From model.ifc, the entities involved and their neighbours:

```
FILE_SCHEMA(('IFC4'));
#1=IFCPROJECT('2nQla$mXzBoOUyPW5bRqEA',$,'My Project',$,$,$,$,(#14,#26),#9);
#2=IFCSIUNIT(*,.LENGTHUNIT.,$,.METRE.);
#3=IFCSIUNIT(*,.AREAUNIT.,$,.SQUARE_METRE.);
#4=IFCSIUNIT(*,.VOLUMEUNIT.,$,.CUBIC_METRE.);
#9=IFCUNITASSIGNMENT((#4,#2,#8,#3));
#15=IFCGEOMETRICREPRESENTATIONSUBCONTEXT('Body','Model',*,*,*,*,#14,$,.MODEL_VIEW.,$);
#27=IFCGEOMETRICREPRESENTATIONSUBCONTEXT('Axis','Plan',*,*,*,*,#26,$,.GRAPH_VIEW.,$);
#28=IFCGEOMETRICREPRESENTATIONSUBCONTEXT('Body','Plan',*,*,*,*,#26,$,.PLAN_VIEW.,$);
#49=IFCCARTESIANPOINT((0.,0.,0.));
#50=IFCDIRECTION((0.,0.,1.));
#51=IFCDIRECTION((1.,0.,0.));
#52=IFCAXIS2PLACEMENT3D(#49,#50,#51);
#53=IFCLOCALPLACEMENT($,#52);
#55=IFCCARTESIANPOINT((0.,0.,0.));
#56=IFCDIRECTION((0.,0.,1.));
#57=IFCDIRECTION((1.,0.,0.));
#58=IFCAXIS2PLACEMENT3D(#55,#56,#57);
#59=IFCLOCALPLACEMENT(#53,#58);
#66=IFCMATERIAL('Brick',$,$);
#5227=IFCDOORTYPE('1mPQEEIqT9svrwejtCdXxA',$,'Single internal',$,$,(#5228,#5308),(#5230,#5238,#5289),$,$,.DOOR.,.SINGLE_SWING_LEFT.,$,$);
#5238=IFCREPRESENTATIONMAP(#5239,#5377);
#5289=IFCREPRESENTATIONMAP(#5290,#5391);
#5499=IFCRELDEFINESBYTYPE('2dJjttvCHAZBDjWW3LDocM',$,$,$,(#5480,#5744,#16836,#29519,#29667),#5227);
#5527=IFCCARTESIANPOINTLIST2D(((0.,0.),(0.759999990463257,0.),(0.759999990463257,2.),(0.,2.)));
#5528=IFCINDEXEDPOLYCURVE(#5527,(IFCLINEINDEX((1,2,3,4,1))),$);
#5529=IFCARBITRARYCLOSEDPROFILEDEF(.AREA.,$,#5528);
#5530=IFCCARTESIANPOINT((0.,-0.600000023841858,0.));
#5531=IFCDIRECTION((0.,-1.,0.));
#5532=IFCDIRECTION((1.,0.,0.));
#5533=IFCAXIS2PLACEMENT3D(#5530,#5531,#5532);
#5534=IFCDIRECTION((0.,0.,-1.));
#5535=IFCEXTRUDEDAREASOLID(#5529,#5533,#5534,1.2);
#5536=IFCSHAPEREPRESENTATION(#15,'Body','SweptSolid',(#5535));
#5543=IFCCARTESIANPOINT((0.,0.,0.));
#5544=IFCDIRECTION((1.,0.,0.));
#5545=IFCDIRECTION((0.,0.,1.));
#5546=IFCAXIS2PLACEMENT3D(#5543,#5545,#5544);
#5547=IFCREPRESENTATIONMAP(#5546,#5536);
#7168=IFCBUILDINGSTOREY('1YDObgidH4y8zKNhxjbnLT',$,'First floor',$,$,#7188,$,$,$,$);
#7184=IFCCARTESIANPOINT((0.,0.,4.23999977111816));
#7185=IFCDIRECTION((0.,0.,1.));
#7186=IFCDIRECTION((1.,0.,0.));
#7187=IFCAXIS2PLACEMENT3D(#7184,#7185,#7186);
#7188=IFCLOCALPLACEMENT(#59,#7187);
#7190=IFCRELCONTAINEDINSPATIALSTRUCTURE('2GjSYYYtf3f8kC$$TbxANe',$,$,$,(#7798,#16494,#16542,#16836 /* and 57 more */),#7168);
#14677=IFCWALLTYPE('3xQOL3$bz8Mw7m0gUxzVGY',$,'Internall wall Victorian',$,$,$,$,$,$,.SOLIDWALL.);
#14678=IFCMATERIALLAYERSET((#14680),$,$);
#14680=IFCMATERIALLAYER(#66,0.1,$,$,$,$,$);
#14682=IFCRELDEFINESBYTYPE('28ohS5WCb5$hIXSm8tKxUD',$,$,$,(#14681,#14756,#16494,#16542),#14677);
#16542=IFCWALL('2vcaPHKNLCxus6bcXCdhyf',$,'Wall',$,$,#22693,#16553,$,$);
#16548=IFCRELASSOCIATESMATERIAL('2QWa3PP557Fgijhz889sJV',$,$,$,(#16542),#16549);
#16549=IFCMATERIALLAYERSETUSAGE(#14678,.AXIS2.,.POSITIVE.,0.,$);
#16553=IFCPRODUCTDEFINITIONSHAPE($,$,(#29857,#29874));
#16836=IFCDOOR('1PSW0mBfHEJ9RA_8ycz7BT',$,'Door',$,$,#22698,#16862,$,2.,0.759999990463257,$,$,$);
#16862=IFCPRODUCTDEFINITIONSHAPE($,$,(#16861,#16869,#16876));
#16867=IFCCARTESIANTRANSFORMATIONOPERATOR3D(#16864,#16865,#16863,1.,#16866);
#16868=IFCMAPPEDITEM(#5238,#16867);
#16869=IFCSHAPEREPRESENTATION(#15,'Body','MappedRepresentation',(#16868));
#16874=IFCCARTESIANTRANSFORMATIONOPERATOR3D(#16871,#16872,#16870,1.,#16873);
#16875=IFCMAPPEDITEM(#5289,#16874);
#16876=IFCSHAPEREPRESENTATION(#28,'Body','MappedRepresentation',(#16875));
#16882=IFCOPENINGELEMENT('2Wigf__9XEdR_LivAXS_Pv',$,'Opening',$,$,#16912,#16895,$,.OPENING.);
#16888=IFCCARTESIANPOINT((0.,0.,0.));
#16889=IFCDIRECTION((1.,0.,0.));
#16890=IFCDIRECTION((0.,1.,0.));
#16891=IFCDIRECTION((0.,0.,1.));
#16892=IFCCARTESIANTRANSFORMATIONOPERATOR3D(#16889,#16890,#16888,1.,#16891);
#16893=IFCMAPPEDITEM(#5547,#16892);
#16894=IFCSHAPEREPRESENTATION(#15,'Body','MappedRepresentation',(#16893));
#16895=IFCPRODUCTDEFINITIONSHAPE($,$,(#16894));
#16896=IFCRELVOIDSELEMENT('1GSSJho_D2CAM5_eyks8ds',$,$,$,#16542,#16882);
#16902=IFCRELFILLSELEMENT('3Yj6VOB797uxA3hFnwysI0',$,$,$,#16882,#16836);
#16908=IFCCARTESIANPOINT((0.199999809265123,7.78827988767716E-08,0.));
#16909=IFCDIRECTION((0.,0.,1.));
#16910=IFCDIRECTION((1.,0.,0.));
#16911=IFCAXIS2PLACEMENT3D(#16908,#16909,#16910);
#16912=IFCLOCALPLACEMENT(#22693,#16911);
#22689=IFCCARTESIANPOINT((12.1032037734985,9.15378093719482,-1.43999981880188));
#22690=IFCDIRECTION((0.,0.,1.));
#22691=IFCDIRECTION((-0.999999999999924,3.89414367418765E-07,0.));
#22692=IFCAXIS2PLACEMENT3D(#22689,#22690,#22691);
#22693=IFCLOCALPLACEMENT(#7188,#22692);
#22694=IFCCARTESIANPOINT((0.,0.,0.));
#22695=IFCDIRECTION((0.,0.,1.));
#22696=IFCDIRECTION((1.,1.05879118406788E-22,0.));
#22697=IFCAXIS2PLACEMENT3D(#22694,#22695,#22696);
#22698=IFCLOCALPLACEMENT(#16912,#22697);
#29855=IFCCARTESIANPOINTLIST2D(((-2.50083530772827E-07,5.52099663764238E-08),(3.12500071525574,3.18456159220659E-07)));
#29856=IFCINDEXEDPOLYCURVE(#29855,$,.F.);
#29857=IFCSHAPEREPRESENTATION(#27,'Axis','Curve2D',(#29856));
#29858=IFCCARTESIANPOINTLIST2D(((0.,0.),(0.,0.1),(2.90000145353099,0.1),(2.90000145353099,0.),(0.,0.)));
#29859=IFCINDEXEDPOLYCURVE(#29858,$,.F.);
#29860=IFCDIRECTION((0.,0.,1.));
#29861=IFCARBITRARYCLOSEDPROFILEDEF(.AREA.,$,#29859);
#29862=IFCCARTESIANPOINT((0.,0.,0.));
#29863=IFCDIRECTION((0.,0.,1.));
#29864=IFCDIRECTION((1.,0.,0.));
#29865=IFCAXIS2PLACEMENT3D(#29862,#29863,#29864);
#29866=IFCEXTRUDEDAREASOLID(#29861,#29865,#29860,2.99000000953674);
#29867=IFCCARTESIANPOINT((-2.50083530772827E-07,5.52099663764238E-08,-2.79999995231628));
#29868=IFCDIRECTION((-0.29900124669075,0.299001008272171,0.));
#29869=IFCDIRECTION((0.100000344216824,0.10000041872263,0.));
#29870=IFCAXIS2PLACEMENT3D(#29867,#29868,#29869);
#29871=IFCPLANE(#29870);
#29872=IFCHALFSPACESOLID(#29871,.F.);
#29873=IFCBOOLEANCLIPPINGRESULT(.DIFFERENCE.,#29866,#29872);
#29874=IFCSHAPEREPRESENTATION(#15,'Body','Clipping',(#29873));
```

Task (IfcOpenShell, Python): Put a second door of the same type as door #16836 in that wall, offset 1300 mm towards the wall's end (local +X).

```python
import ifcopenshell
import ifcopenshell.api.feature
import ifcopenshell.api.geometry
import ifcopenshell.api.root
import ifcopenshell.geom
import ifcopenshell.util.element
import ifcopenshell.util.placement
import ifcopenshell.util.shape
import ifcopenshell.util.unit

model = ifcopenshell.open("model.ifc")
unit_scale = ifcopenshell.util.unit.calculate_unit_scale(model)
settings = ifcopenshell.geom.settings()


def volume(element):
    """Net volume in cubic metres, openings subtracted."""
    shape = ifcopenshell.geom.create_shape(settings, element)
    return ifcopenshell.util.shape.get_volume(shape.geometry)


door = model.by_id(16836)
opening = door.FillsVoids[0].RelatingOpeningElement
wall = opening.VoidsElements[0].RelatingBuildingElement
before = volume(wall)
shift = ifcopenshell.util.placement.get_local_placement(wall.ObjectPlacement)[:3, 0] * 1.3 / unit_scale

# copy_class copies the void relationship, type, container and properties, but no geometry.
new_opening = ifcopenshell.api.root.copy_class(model, product=opening)
new_opening.Representation = ifcopenshell.util.element.copy_deep(
    model, opening.Representation, exclude=["IfcGeometricRepresentationContext", "IfcRepresentationMap"]
)
new_door = ifcopenshell.api.root.copy_class(model, product=door)
new_door.Representation = ifcopenshell.util.element.copy_deep(
    model, door.Representation, exclude=["IfcGeometricRepresentationContext", "IfcRepresentationMap"]
)
ifcopenshell.api.feature.add_filling(model, opening=new_opening, element=new_door)

for old, new in ((opening, new_opening), (door, new_door)):
    matrix = ifcopenshell.util.placement.get_local_placement(old.ObjectPlacement)
    matrix[:3, 3] += shift
    ifcopenshell.api.geometry.edit_object_placement(model, product=new, matrix=matrix, is_si=False)

after = volume(wall)

print(f"wall volume {before:.3f} -> {after:.3f} m3")

model.write("model-out.ifc")
```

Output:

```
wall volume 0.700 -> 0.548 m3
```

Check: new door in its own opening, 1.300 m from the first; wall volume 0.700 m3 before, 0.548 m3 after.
